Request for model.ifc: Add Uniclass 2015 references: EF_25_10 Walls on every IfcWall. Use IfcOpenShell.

First a look at what the model holds.

```python
import ifcopenshell

model = ifcopenshell.open("model.ifc")
print(model.schema)
print("classifications:", [c.Name for c in model.by_type("IfcClassification")])
for ifc_class in ("IfcDoor", "IfcRoof", "IfcStair", "IfcWall", "IfcWindow"):
    print(ifc_class, len(model.by_type(ifc_class)))
```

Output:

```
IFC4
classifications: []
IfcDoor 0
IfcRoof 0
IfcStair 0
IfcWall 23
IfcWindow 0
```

```python
import ifcopenshell
import ifcopenshell.api.classification

model = ifcopenshell.open("model.ifc")

system = ifcopenshell.api.classification.add_classification(model, classification="Uniclass 2015")

codes = {
    "IfcWall": ("EF_25_10", "Walls"),
}
for ifc_class, (code, name) in codes.items():
    products = model.by_type(ifc_class)
    ifcopenshell.api.classification.add_reference(
        model, products=products, classification=system, identification=code, name=name
    )
    print(code, len(products))

model.write("model-out.ifc")
```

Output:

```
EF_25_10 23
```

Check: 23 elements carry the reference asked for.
